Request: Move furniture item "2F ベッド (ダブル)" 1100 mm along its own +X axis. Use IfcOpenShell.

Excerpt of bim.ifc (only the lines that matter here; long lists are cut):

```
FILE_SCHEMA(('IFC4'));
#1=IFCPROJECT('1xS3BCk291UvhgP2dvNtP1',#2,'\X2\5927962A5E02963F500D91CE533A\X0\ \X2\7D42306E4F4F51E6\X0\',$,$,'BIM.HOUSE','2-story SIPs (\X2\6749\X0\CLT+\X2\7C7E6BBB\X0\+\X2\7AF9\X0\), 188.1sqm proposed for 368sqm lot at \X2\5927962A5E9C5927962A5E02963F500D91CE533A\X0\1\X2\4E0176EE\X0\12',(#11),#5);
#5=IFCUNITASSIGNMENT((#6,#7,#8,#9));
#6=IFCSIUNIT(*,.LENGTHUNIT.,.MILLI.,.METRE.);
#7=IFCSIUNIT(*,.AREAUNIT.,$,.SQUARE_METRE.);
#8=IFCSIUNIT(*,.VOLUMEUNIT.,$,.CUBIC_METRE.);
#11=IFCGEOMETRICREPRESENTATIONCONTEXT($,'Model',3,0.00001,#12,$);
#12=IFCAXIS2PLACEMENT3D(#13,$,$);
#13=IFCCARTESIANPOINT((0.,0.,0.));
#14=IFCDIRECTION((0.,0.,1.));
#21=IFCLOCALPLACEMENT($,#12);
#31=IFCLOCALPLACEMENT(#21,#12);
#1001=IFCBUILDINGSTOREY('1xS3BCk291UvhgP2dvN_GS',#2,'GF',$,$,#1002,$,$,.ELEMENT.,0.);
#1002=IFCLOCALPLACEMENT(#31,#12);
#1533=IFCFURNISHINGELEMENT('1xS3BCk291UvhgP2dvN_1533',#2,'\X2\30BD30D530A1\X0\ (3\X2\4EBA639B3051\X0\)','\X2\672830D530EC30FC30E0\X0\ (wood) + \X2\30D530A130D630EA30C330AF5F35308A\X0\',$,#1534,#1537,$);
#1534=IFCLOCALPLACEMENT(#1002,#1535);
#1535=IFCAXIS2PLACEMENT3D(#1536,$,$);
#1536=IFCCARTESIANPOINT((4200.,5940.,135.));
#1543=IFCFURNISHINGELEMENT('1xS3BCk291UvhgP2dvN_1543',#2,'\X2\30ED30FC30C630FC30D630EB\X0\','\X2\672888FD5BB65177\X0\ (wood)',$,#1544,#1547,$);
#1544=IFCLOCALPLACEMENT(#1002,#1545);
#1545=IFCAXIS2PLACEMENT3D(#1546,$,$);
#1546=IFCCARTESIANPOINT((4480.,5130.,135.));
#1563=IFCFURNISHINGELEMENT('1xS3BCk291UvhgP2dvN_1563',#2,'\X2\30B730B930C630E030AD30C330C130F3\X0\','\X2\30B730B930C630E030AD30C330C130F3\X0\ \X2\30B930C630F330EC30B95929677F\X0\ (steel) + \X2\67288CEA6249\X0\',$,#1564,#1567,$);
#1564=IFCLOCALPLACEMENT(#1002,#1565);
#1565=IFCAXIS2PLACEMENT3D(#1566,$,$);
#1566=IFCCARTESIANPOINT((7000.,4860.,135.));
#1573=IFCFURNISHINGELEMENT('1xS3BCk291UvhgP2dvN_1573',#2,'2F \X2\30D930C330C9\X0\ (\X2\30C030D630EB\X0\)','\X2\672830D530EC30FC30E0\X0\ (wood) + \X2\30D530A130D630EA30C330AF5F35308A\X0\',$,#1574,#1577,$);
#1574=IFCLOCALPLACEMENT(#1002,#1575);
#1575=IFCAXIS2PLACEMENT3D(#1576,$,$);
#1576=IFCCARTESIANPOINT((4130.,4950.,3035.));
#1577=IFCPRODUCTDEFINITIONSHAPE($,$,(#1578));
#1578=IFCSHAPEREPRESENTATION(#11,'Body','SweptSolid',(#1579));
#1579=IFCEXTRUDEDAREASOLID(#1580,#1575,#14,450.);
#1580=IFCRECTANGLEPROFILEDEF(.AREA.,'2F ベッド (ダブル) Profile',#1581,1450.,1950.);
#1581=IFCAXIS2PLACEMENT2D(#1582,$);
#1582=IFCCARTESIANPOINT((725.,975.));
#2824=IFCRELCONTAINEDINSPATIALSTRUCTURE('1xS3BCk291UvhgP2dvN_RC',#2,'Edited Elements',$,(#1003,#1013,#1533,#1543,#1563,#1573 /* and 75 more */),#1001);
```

```python
import ifcopenshell
import ifcopenshell.api.geometry
import ifcopenshell.util.placement
import ifcopenshell.util.unit

model = ifcopenshell.open("bim.ifc")
unit_scale = ifcopenshell.util.unit.calculate_unit_scale(model)

item = model.by_guid("1xS3BCk291UvhgP2dvN_1573")
matrix = ifcopenshell.util.placement.get_local_placement(item.ObjectPlacement)
matrix[:3, 3] += matrix[:3, 0] * 1.1 / unit_scale
ifcopenshell.api.geometry.edit_object_placement(model, product=item, matrix=matrix, is_si=False)

print(ifcopenshell.util.placement.get_local_placement(item.ObjectPlacement).round(3) + 0.0)

model.write("bim_v2.ifc")
```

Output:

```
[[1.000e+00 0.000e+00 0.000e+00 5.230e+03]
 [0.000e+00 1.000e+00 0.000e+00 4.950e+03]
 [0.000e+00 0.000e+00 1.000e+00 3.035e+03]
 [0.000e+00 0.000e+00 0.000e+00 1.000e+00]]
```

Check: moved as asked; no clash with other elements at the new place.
